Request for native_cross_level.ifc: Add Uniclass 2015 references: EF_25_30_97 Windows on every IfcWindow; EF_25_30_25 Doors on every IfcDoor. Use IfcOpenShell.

First a look at what the model holds.

```python
import ifcopenshell

model = ifcopenshell.open("native_cross_level.ifc")
print(model.schema)
print("classifications:", [c.Name for c in model.by_type("IfcClassification")])
for ifc_class in ("IfcDoor", "IfcRoof", "IfcStair", "IfcWall", "IfcWindow"):
    print(ifc_class, len(model.by_type(ifc_class)))
```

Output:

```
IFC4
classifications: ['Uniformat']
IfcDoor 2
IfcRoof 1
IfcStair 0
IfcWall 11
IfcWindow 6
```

```python
import ifcopenshell
import ifcopenshell.api.classification

model = ifcopenshell.open("native_cross_level.ifc")

system = ifcopenshell.api.classification.add_classification(model, classification="Uniclass 2015")

codes = {
    "IfcWindow": ("EF_25_30_97", "Windows"),
    "IfcDoor": ("EF_25_30_25", "Doors"),
}
for ifc_class, (code, name) in codes.items():
    products = model.by_type(ifc_class)
    ifcopenshell.api.classification.add_reference(
        model, products=products, classification=system, identification=code, name=name
    )
    print(code, len(products))

model.write("native_cross_level_edited.ifc")
```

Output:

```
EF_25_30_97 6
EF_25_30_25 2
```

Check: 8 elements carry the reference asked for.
